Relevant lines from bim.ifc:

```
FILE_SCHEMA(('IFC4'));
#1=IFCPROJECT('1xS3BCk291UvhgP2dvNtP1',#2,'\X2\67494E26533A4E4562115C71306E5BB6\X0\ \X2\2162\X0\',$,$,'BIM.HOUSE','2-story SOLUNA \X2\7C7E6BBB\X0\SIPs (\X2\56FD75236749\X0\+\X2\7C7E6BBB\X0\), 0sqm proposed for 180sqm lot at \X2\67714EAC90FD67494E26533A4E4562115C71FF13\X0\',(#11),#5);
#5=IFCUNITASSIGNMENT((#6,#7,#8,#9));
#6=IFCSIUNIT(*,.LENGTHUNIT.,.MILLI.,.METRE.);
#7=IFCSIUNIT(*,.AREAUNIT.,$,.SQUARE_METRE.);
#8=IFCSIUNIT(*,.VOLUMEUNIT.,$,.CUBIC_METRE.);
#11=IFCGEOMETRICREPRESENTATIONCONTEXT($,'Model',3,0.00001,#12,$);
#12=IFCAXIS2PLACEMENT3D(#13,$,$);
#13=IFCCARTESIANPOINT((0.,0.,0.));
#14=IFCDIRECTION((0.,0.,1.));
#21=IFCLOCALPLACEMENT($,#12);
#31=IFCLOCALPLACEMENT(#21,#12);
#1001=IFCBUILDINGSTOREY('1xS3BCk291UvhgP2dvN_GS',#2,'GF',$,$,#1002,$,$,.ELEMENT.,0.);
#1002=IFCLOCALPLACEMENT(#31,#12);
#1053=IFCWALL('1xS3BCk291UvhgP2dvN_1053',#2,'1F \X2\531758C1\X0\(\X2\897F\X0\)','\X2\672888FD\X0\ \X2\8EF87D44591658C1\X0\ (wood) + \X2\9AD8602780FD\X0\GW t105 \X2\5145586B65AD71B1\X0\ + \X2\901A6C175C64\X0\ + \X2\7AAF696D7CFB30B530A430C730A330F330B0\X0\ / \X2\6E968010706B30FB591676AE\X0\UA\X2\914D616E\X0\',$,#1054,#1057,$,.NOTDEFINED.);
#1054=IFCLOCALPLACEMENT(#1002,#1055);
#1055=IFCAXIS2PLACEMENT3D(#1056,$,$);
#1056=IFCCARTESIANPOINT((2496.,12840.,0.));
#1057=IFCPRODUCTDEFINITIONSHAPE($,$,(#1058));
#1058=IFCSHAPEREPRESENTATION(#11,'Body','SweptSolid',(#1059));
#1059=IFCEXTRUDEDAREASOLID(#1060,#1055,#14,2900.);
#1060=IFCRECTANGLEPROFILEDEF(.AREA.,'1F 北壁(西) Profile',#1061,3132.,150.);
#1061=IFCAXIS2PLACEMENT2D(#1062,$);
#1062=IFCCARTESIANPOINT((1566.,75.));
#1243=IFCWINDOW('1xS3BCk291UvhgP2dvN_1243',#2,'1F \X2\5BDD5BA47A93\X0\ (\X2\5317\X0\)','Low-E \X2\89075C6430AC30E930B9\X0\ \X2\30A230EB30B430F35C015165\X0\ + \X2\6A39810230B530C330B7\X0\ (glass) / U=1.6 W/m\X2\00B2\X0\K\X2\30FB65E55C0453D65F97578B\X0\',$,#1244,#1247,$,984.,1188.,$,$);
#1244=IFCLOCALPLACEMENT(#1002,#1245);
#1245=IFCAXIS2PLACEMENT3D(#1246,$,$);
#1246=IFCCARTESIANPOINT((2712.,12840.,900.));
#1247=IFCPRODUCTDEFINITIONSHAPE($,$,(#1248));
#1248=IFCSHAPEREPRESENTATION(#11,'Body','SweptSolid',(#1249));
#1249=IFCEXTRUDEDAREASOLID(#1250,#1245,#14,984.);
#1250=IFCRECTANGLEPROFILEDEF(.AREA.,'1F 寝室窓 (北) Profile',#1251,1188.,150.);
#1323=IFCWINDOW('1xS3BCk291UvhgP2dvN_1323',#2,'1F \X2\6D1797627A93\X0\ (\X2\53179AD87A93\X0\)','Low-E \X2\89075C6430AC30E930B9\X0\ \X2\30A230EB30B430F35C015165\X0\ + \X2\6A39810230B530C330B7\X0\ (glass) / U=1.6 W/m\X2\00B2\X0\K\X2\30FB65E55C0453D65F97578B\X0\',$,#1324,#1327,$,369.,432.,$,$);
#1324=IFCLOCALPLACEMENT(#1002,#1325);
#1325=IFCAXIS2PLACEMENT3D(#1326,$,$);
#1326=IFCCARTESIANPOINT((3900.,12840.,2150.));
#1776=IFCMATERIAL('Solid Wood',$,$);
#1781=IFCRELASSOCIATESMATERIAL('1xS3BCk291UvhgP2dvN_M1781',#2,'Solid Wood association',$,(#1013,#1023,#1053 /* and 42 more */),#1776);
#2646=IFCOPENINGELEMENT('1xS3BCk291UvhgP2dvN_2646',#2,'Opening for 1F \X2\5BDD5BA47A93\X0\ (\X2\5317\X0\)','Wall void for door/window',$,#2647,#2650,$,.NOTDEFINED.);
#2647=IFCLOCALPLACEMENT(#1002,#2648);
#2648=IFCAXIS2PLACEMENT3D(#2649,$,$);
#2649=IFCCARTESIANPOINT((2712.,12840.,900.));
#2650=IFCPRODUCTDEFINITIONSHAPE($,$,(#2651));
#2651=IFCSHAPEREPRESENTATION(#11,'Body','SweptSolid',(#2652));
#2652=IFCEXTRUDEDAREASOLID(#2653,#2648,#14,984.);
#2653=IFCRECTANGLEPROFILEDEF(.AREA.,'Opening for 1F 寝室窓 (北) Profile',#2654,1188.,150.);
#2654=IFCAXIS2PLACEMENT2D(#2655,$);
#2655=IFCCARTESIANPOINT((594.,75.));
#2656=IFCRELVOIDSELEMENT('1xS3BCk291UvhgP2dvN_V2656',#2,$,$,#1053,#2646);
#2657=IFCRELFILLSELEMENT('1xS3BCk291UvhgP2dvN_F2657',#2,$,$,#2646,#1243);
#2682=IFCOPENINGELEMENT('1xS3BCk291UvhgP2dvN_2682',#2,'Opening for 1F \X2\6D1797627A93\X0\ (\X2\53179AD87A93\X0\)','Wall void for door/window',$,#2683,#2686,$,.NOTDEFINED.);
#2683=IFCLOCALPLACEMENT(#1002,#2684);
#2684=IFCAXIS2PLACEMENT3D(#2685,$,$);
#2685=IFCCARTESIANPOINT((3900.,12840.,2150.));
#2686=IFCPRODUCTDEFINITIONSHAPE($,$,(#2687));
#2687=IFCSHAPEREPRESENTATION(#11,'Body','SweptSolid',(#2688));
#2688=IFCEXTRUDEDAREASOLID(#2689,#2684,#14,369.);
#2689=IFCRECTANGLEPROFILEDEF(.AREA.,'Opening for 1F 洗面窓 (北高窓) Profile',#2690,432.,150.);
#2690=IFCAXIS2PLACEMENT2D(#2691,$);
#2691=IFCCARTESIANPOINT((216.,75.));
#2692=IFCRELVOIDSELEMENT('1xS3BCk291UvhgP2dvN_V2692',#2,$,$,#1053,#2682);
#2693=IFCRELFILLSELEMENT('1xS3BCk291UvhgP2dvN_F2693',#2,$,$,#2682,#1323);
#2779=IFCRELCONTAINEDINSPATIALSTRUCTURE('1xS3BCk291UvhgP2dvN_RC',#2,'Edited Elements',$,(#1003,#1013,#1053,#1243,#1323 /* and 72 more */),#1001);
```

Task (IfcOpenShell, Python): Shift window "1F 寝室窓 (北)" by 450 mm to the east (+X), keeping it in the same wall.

```python
import ifcopenshell
import ifcopenshell.api.geometry
import ifcopenshell.util.placement
import ifcopenshell.util.unit

model = ifcopenshell.open("bim.ifc")
unit_scale = ifcopenshell.util.unit.calculate_unit_scale(model)

window = model.by_guid("1xS3BCk291UvhgP2dvN_1243")
opening = window.FillsVoids[0].RelatingOpeningElement
wall = opening.VoidsElements[0].RelatingBuildingElement

wall_matrix = ifcopenshell.util.placement.get_local_placement(wall.ObjectPlacement)
shift = wall_matrix[:3, 0] * 0.45 / unit_scale
before = ifcopenshell.util.placement.get_local_placement(window.ObjectPlacement)[:3, 3].copy()

# The window is not placed relative to its opening, so move both.
for product in (opening, window):
    matrix = ifcopenshell.util.placement.get_local_placement(product.ObjectPlacement)
    matrix[:3, 3] += shift
    ifcopenshell.api.geometry.edit_object_placement(model, product=product, matrix=matrix, is_si=False)

after = ifcopenshell.util.placement.get_local_placement(window.ObjectPlacement)[:3, 3]
print("window moved by", (after - before).round(3) + 0.0)

model.write("bim_edited.ifc")
```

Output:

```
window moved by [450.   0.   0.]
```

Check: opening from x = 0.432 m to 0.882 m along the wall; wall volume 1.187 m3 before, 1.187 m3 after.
